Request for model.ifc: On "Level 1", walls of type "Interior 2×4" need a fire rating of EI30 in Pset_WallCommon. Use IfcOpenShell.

First a look at what the model holds.

```python
import ifcopenshell
import ifcopenshell.util.element

model = ifcopenshell.open("model.ifc")
print(model.schema)
storey = next(s for s in model.by_type("IfcBuildingStorey") if s.Name == "Level 1")
walls = [e for e in ifcopenshell.util.element.get_decomposition(storey) if e.is_a("IfcWall")]
seen = {}
for e in walls:
    element_type = ifcopenshell.util.element.get_type(e)
    key = (element_type.Name if element_type != e and element_type else None, ifcopenshell.util.element.get_pset(e, "Pset_WallCommon", "FireRating"))
    seen[key] = seen.get(key, 0) + 1
for (name, value), count in sorted(seen.items(), key=str):
    print(count, "x", name, "|", value)
```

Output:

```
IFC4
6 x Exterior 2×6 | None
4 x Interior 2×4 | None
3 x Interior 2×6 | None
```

```python
import ifcopenshell
import ifcopenshell.api.pset
import ifcopenshell.util.element

model = ifcopenshell.open("model.ifc")

storey = next(s for s in model.by_type("IfcBuildingStorey") if s.Name == "Level 1")
walls = [e for e in ifcopenshell.util.element.get_decomposition(storey) if e.is_a("IfcWall")]

count = 0
for e in walls:
    element_type = ifcopenshell.util.element.get_type(e)
    if element_type in (None, e) or element_type.Name != "Interior 2×4":
        continue
    # add_pset returns the element's existing set when there is one.
    pset = ifcopenshell.api.pset.add_pset(model, product=e, name="Pset_WallCommon")
    ifcopenshell.api.pset.edit_pset(model, pset=pset, properties={"FireRating": "EI30"})
    count += 1

print(count, "walls updated")

model.write("model_edited.ifc")
```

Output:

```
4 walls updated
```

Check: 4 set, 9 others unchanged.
